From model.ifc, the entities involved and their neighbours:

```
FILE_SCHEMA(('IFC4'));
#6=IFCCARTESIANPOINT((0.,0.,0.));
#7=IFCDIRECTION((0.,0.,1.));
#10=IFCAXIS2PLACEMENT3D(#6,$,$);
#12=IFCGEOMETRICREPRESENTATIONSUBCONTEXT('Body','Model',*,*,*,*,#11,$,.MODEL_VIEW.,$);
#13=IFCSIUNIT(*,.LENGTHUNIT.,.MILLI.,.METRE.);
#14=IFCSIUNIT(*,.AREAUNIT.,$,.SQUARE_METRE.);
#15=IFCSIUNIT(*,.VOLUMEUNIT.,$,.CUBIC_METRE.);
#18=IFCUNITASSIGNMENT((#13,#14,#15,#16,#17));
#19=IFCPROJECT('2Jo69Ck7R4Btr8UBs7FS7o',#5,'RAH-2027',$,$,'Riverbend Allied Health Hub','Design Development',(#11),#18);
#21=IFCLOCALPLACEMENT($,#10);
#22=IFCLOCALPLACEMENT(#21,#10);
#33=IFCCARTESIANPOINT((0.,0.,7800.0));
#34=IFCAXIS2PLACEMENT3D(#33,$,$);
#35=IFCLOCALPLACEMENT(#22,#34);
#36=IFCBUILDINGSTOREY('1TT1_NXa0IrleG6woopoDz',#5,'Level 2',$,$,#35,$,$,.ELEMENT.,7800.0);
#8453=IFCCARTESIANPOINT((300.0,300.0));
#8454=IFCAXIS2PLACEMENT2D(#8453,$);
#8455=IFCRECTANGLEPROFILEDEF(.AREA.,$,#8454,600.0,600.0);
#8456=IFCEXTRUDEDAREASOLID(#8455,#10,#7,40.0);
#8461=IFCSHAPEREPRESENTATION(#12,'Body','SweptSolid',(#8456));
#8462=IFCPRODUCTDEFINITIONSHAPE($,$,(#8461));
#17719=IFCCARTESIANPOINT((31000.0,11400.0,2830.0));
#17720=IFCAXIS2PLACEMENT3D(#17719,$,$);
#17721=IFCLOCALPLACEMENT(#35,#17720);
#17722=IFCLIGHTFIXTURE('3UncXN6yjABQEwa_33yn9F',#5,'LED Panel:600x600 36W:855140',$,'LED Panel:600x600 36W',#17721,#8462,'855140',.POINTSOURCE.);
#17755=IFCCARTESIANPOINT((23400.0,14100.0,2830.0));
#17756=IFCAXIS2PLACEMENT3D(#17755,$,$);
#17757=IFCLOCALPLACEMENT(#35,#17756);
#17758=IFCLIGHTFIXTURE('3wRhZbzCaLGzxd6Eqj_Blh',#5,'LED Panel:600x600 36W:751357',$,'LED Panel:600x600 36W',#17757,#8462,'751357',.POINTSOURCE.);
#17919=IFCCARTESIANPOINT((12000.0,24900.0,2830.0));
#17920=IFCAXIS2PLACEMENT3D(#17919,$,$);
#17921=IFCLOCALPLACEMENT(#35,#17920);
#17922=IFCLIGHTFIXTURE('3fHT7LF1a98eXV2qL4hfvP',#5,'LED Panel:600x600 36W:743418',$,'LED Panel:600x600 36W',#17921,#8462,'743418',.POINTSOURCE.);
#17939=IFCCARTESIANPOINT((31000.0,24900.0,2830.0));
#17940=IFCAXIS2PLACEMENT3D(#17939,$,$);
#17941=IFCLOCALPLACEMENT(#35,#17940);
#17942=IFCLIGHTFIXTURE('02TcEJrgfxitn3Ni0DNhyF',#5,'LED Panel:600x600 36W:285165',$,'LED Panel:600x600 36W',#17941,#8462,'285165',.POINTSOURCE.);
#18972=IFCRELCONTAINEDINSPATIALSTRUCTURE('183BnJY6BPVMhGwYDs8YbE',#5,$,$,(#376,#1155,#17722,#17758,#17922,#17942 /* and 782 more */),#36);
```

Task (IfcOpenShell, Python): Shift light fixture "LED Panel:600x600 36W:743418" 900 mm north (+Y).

```python
import ifcopenshell
import ifcopenshell.api.geometry
import ifcopenshell.util.placement

model = ifcopenshell.open("model.ifc")

item = model.by_guid("3fHT7LF1a98eXV2qL4hfvP")
matrix = ifcopenshell.util.placement.get_local_placement(item.ObjectPlacement)
matrix[1, 3] += 900.0
ifcopenshell.api.geometry.edit_object_placement(model, product=item, matrix=matrix, is_si=False)

print(ifcopenshell.util.placement.get_local_placement(item.ObjectPlacement).round(3) + 0.0)

model.write("model_edited.ifc")
```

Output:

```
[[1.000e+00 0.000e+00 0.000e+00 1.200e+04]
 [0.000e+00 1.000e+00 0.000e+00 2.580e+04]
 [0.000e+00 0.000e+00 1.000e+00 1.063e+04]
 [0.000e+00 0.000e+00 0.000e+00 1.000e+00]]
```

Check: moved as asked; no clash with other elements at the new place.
